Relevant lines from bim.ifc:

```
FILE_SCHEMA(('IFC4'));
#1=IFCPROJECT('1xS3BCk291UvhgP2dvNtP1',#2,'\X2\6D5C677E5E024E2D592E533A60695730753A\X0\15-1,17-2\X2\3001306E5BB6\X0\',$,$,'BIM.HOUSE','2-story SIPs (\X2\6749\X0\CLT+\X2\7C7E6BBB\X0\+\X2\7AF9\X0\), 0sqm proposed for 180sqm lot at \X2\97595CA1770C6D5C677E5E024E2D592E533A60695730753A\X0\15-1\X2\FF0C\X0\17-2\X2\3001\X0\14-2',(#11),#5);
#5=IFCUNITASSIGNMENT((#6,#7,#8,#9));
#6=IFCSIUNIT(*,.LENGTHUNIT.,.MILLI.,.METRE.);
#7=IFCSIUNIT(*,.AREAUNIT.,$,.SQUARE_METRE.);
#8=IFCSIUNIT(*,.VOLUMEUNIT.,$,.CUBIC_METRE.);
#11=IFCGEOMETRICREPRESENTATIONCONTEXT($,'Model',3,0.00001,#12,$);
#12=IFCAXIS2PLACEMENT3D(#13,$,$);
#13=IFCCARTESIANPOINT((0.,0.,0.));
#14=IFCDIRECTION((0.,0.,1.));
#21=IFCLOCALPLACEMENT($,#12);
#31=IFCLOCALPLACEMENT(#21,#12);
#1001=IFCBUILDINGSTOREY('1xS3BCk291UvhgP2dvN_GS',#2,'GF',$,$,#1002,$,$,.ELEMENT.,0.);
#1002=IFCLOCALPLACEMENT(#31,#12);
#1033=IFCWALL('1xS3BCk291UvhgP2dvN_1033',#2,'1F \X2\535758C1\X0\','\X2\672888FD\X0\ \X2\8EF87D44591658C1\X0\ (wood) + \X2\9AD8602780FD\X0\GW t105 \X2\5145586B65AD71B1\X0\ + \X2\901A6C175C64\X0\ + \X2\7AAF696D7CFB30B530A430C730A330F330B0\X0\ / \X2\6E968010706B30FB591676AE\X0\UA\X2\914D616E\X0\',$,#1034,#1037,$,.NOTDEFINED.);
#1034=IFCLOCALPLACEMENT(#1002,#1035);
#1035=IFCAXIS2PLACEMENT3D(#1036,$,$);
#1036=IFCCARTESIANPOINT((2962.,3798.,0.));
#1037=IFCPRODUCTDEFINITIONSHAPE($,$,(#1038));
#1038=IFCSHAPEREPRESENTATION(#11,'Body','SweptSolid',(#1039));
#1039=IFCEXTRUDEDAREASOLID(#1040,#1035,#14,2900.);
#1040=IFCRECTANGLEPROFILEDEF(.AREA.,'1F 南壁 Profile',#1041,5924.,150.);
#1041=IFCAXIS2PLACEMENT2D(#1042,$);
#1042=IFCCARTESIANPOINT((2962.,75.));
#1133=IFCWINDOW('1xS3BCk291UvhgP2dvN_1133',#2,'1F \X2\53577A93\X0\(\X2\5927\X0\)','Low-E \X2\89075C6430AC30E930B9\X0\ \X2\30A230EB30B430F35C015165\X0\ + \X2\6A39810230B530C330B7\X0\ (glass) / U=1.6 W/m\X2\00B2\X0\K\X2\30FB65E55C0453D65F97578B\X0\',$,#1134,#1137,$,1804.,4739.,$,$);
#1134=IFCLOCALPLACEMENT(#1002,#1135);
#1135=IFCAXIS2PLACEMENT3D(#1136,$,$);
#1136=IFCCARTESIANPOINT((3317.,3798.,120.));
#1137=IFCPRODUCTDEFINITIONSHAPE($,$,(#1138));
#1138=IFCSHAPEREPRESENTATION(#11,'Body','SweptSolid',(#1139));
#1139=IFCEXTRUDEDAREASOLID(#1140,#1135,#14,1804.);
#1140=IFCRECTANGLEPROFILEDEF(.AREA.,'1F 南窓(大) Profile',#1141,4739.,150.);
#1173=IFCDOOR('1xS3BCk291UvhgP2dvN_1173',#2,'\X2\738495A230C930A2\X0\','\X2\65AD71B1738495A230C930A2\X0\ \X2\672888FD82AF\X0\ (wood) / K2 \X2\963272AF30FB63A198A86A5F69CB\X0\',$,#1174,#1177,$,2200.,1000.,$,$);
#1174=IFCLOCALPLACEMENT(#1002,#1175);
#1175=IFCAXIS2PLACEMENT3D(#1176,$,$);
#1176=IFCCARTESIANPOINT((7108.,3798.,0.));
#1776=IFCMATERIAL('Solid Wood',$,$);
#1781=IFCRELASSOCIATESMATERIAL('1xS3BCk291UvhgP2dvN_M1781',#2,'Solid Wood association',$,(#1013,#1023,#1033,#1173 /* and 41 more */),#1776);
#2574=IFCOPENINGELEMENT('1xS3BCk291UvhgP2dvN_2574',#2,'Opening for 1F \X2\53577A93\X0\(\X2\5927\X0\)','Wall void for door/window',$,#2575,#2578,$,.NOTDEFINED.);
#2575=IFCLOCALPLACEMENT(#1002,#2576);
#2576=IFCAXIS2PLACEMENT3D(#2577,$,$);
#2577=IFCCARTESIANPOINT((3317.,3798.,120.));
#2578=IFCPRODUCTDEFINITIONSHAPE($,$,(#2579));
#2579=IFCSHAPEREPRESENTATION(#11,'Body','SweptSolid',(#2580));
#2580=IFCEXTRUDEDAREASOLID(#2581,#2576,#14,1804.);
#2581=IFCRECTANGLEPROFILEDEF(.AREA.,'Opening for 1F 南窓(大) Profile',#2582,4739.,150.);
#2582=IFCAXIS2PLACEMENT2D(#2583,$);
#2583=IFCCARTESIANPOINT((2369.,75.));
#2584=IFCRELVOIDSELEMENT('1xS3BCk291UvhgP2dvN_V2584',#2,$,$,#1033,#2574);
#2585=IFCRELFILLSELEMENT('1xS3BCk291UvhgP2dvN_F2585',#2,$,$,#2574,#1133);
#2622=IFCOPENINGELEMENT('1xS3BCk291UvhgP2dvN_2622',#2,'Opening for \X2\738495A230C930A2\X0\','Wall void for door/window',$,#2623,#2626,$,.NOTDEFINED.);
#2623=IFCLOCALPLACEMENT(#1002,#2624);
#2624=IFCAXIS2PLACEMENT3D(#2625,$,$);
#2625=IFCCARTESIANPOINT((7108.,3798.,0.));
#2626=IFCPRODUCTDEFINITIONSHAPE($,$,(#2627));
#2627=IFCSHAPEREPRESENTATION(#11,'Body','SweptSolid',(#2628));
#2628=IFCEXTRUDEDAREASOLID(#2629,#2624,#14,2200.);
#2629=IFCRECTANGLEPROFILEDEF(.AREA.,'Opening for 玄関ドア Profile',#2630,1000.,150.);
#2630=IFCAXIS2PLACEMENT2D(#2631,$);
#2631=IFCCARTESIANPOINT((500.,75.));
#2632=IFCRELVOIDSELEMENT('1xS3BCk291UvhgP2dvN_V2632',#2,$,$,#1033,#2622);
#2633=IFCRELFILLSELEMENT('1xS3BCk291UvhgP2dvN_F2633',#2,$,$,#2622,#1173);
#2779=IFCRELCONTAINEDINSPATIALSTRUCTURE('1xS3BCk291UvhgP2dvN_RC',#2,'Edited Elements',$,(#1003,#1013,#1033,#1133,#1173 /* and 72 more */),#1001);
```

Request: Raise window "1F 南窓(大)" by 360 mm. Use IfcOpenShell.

```python
import numpy as np
import ifcopenshell
import ifcopenshell.api.geometry
import ifcopenshell.util.placement
import ifcopenshell.util.unit

model = ifcopenshell.open("bim.ifc")
unit_scale = ifcopenshell.util.unit.calculate_unit_scale(model)

window = model.by_guid("1xS3BCk291UvhgP2dvN_1133")
opening = window.FillsVoids[0].RelatingOpeningElement
dz = 360.0

shift = np.array([0.0, 0.0, dz])
# The window is not placed relative to its opening, so move both.
for product in (opening, window):
    matrix = ifcopenshell.util.placement.get_local_placement(product.ObjectPlacement)
    matrix[:3, 3] += shift
    ifcopenshell.api.geometry.edit_object_placement(model, product=product, matrix=matrix, is_si=False)

print(f"moved by {dz * unit_scale:+.3f} m")

model.write("bim-out.ifc")
```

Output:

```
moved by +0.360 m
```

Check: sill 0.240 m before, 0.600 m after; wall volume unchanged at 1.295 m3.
